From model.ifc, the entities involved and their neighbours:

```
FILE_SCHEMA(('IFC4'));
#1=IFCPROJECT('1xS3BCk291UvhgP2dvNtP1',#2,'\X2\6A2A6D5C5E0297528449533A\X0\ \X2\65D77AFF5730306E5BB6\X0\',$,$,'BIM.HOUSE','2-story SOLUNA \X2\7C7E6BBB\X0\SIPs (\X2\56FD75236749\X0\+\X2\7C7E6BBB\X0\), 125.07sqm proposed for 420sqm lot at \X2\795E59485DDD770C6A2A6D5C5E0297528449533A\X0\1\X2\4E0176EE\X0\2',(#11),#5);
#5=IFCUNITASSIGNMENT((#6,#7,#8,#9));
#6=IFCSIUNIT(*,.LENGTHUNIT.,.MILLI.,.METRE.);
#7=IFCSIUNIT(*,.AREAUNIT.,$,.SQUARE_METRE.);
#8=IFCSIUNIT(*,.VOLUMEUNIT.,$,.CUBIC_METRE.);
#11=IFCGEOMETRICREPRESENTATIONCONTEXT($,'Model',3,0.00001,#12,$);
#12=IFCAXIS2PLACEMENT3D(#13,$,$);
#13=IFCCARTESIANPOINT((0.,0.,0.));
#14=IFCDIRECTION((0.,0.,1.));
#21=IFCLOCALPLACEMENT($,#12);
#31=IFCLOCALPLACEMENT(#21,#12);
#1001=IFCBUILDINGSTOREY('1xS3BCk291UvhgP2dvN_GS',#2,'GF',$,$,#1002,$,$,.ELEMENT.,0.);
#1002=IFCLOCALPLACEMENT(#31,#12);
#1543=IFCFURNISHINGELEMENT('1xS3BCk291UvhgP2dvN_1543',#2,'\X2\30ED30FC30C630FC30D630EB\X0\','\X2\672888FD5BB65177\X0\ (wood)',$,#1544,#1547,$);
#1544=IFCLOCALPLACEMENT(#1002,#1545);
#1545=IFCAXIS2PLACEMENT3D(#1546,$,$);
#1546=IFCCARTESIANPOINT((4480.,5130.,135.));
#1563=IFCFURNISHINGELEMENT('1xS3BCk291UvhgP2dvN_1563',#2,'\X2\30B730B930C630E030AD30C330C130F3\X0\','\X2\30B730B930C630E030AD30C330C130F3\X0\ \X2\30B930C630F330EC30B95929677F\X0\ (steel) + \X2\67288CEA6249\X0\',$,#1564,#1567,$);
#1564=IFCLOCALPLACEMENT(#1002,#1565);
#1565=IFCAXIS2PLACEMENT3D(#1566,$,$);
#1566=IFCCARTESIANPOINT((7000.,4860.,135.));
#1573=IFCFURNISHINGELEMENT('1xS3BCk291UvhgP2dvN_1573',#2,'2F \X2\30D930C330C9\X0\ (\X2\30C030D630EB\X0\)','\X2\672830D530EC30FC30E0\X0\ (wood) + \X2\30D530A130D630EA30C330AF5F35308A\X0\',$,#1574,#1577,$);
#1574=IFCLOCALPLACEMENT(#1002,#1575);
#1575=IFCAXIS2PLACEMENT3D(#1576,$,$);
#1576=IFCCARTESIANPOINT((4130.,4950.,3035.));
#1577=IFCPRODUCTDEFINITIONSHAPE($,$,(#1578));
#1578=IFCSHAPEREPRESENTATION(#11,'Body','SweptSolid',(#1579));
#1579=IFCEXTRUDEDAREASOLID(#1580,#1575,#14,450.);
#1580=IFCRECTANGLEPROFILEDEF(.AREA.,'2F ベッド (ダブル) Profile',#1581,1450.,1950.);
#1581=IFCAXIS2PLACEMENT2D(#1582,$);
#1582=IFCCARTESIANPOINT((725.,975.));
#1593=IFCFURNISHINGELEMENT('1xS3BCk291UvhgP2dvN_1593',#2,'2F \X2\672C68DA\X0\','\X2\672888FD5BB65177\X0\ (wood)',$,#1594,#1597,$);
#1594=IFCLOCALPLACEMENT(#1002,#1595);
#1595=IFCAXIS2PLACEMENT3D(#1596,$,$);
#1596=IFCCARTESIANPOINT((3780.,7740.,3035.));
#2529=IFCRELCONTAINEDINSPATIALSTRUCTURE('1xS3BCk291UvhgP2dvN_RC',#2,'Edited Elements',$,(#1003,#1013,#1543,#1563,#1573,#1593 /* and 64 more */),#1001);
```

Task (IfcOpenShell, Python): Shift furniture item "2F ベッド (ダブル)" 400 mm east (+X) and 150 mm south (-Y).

```python
import ifcopenshell
import ifcopenshell.api.geometry
import ifcopenshell.util.placement

model = ifcopenshell.open("model.ifc")

item = model.by_guid("1xS3BCk291UvhgP2dvN_1573")
matrix = ifcopenshell.util.placement.get_local_placement(item.ObjectPlacement)
matrix[0, 3] += 400.0
matrix[1, 3] -= 150.0
ifcopenshell.api.geometry.edit_object_placement(model, product=item, matrix=matrix, is_si=False)

print(ifcopenshell.util.placement.get_local_placement(item.ObjectPlacement).round(3) + 0.0)

model.write("model-out.ifc")
```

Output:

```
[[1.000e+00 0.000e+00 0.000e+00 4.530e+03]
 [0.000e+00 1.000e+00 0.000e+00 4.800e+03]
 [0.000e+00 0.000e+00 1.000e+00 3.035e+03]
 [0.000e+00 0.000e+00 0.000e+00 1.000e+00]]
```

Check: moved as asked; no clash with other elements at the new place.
